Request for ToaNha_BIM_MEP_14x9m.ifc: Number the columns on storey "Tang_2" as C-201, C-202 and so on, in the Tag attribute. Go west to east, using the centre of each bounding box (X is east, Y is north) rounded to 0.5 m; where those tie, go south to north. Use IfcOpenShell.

First a look at what the model holds.

```python
import ifcopenshell
import ifcopenshell.util.element
import ifcopenshell.util.placement

model = ifcopenshell.open("ToaNha_BIM_MEP_14x9m.ifc")
print(model.schema)
storey = next(s for s in model.by_type("IfcBuildingStorey") if s.Name == "Tang_2")
columns = [e for e in ifcopenshell.util.element.get_decomposition(storey) if e.is_a("IfcColumn")]
for e in sorted(columns, key=lambda e: e.id()):
    origin = ifcopenshell.util.placement.get_local_placement(e.ObjectPlacement)[:3, 3]
    print(e.id(), e.Tag, e.Name, origin.round(2) + 0.0, sep=" | ")
```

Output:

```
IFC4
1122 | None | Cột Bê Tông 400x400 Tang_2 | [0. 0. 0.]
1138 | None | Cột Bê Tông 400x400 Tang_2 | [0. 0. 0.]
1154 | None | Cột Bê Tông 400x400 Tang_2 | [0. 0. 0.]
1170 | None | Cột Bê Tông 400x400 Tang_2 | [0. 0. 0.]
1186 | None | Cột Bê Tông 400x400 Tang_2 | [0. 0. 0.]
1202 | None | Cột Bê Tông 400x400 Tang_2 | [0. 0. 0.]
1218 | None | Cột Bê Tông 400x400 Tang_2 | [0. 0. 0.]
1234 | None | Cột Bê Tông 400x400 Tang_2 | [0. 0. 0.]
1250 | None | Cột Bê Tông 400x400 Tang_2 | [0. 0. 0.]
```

```python
import ifcopenshell
import ifcopenshell.geom
import ifcopenshell.util.element
import ifcopenshell.util.shape

model = ifcopenshell.open("ToaNha_BIM_MEP_14x9m.ifc")
settings = ifcopenshell.geom.settings()
settings.set("use-world-coords", True)


def centre(element):
    shape = ifcopenshell.geom.create_shape(settings, element)
    return ifcopenshell.util.shape.get_bbox_centroid(shape.geometry)


storey = next(s for s in model.by_type("IfcBuildingStorey") if s.Name == "Tang_2")
columns = [e for e in ifcopenshell.util.element.get_decomposition(storey) if e.is_a("IfcColumn")]

# Insertion points can sit at a corner or the storey origin, so sort by the geometry (in metres).
centres = {e: centre(e) for e in columns}
columns.sort(key=lambda e: (round(centres[e][0] / 0.5), centres[e][1]))

for i, e in enumerate(columns, start=1):
    number = f"C-2{i:02d}"
    e.Tag = number
    print(e.id(), number)

model.write("ToaNha_BIM_MEP_14x9m_edited.ifc")
```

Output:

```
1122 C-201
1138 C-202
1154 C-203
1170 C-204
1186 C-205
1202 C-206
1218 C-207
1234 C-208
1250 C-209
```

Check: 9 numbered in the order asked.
